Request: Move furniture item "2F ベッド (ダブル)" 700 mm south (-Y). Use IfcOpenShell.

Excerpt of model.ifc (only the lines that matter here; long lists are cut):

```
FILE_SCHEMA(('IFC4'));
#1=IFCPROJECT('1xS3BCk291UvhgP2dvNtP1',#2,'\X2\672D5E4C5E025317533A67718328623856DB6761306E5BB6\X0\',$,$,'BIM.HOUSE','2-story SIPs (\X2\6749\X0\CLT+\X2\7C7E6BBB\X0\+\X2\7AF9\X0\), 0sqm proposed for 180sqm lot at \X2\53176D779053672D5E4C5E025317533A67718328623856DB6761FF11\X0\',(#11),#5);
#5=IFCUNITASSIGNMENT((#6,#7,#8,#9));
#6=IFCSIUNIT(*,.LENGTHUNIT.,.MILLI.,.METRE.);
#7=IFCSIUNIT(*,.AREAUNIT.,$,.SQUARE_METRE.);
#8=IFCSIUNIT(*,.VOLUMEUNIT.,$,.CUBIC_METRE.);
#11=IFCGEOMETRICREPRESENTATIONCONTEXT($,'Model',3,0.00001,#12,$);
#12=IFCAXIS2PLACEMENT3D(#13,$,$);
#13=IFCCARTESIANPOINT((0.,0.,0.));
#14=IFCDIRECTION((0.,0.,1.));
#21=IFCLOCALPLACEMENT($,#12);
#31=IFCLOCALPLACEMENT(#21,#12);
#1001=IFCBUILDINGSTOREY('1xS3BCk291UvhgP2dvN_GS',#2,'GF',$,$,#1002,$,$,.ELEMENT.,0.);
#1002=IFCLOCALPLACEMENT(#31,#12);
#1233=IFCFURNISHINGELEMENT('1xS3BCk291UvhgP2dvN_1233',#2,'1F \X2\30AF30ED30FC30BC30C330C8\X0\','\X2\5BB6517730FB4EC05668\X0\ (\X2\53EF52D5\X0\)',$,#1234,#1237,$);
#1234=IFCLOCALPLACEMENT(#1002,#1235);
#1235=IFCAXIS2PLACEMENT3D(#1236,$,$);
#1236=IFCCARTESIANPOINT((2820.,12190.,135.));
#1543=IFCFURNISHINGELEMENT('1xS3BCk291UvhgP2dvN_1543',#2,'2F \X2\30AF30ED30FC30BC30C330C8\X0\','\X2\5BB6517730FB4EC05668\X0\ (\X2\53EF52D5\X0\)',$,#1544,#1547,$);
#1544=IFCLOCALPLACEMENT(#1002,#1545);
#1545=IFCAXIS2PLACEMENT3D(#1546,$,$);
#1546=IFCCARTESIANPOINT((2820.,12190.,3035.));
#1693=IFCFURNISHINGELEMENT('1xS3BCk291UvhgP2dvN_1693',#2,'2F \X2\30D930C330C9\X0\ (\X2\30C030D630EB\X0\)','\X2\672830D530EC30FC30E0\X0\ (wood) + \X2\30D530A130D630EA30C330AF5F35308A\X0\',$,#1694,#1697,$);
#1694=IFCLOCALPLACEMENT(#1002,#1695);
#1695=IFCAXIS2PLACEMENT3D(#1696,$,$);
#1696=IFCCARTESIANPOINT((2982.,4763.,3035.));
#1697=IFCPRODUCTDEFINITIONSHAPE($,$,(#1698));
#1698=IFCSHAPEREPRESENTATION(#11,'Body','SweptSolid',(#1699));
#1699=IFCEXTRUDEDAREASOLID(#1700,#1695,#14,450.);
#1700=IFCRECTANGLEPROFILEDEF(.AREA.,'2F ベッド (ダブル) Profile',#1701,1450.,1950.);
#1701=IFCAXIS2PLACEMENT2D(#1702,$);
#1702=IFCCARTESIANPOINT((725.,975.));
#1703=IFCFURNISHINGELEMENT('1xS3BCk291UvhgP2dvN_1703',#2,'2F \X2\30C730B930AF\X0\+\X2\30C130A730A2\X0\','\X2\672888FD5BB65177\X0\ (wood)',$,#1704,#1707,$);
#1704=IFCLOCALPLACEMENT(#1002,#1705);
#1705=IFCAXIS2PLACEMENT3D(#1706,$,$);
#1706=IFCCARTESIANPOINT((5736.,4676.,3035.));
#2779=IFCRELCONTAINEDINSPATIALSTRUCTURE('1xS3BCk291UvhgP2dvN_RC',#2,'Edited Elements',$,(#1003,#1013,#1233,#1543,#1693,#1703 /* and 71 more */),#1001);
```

```python
import ifcopenshell
import ifcopenshell.api.geometry
import ifcopenshell.util.placement
import ifcopenshell.util.unit

model = ifcopenshell.open("model.ifc")
unit_scale = ifcopenshell.util.unit.calculate_unit_scale(model)

item = model.by_guid("1xS3BCk291UvhgP2dvN_1693")
matrix = ifcopenshell.util.placement.get_local_placement(item.ObjectPlacement)
matrix[1, 3] -= 0.7 / unit_scale
ifcopenshell.api.geometry.edit_object_placement(model, product=item, matrix=matrix, is_si=False)

print(ifcopenshell.util.placement.get_local_placement(item.ObjectPlacement).round(3) + 0.0)

model.write("model_v2.ifc")
```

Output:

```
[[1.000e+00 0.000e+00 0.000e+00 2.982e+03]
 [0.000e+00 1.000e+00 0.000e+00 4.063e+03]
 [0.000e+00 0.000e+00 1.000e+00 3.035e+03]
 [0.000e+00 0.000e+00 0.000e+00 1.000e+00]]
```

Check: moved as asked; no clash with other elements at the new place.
